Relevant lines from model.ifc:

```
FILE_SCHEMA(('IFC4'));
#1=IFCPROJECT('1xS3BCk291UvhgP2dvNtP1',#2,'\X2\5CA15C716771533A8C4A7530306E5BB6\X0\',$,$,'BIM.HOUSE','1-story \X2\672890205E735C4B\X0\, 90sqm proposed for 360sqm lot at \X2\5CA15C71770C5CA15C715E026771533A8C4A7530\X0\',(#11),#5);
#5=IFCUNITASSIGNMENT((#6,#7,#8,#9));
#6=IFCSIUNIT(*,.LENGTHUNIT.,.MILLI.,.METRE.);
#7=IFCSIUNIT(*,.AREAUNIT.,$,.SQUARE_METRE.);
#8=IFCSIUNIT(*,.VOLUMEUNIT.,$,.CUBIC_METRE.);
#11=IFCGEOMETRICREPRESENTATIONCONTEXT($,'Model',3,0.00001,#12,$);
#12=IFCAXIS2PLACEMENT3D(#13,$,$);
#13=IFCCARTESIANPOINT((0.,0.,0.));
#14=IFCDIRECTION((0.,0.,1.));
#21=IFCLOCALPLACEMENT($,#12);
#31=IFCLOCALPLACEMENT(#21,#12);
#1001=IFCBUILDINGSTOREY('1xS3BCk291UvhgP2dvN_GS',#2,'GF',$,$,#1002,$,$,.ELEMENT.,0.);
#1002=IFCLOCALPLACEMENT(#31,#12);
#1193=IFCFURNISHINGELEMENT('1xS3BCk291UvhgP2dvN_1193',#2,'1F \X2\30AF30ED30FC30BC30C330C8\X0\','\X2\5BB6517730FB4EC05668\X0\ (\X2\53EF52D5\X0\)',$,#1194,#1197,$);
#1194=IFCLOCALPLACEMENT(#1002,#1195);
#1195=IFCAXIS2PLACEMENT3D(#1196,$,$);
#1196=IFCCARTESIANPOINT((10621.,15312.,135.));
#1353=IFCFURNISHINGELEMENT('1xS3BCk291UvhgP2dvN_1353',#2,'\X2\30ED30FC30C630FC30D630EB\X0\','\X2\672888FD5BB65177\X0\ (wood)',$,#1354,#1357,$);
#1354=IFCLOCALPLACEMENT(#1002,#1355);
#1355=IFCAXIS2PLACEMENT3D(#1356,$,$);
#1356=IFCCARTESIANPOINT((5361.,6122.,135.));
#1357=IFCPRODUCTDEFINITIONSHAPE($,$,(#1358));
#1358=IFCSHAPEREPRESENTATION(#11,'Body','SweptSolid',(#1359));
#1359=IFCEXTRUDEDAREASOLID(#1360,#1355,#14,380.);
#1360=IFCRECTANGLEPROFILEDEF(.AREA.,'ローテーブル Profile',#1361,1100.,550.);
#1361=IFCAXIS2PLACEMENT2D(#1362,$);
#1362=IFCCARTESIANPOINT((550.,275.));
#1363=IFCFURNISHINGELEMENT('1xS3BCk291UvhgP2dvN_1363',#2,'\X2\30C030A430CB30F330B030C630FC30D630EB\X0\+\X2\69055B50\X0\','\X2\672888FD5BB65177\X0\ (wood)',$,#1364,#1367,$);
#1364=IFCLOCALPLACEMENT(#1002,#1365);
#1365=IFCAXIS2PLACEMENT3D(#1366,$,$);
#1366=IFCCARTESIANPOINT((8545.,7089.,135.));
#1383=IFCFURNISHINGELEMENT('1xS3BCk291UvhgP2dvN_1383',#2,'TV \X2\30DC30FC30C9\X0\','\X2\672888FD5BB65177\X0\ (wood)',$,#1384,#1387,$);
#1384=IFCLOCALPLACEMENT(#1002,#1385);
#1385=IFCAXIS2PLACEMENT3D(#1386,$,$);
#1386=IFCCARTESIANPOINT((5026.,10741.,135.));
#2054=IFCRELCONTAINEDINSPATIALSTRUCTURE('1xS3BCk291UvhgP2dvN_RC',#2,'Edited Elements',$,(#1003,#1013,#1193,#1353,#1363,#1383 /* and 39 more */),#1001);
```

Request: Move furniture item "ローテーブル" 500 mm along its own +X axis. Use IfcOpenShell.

```python
import ifcopenshell
import ifcopenshell.api.geometry
import ifcopenshell.util.placement

model = ifcopenshell.open("model.ifc")

item = model.by_guid("1xS3BCk291UvhgP2dvN_1353")
matrix = ifcopenshell.util.placement.get_local_placement(item.ObjectPlacement)
matrix[:3, 3] += matrix[:3, 0] * 500.0
ifcopenshell.api.geometry.edit_object_placement(model, product=item, matrix=matrix, is_si=False)

print(ifcopenshell.util.placement.get_local_placement(item.ObjectPlacement).round(3) + 0.0)

model.write("model_v2.ifc")
```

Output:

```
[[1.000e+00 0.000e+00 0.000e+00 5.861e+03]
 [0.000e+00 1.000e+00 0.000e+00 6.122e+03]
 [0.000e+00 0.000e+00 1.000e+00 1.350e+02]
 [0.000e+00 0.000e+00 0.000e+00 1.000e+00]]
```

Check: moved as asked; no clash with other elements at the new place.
